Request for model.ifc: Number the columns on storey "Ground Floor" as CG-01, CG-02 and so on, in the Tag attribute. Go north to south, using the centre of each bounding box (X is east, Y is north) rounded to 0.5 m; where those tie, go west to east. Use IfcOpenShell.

First a look at what the model holds.

```python
import ifcopenshell
import ifcopenshell.util.element
import ifcopenshell.util.placement

model = ifcopenshell.open("model.ifc")
print(model.schema)
storey = next(s for s in model.by_type("IfcBuildingStorey") if s.Name == "Ground Floor")
columns = [e for e in ifcopenshell.util.element.get_decomposition(storey) if e.is_a("IfcColumn")]
for e in sorted(columns, key=lambda e: e.id()):
    origin = ifcopenshell.util.placement.get_local_placement(e.ObjectPlacement)[:3, 3]
    print(e.id(), e.Tag, e.Name, origin.round(2) + 0.0, sep=" | ")
```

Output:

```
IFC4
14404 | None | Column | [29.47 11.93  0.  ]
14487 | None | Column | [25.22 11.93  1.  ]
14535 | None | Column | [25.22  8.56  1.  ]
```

```python
import ifcopenshell
import ifcopenshell.geom
import ifcopenshell.util.element
import ifcopenshell.util.shape

model = ifcopenshell.open("model.ifc")
settings = ifcopenshell.geom.settings()
settings.set("use-world-coords", True)


def centre(element):
    shape = ifcopenshell.geom.create_shape(settings, element)
    return ifcopenshell.util.shape.get_bbox_centroid(shape.geometry)


storey = next(s for s in model.by_type("IfcBuildingStorey") if s.Name == "Ground Floor")
columns = [e for e in ifcopenshell.util.element.get_decomposition(storey) if e.is_a("IfcColumn")]

# Insertion points can sit at a corner or the storey origin, so sort by the geometry (in metres).
centres = {e: centre(e) for e in columns}
columns.sort(key=lambda e: (-round(centres[e][1] / 0.5), centres[e][0]))

for i, e in enumerate(columns, start=1):
    number = f"CG-{i:02d}"
    e.Tag = number
    print(e.id(), number)

model.write("model-out.ifc")
```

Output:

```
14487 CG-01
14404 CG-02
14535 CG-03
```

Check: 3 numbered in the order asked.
